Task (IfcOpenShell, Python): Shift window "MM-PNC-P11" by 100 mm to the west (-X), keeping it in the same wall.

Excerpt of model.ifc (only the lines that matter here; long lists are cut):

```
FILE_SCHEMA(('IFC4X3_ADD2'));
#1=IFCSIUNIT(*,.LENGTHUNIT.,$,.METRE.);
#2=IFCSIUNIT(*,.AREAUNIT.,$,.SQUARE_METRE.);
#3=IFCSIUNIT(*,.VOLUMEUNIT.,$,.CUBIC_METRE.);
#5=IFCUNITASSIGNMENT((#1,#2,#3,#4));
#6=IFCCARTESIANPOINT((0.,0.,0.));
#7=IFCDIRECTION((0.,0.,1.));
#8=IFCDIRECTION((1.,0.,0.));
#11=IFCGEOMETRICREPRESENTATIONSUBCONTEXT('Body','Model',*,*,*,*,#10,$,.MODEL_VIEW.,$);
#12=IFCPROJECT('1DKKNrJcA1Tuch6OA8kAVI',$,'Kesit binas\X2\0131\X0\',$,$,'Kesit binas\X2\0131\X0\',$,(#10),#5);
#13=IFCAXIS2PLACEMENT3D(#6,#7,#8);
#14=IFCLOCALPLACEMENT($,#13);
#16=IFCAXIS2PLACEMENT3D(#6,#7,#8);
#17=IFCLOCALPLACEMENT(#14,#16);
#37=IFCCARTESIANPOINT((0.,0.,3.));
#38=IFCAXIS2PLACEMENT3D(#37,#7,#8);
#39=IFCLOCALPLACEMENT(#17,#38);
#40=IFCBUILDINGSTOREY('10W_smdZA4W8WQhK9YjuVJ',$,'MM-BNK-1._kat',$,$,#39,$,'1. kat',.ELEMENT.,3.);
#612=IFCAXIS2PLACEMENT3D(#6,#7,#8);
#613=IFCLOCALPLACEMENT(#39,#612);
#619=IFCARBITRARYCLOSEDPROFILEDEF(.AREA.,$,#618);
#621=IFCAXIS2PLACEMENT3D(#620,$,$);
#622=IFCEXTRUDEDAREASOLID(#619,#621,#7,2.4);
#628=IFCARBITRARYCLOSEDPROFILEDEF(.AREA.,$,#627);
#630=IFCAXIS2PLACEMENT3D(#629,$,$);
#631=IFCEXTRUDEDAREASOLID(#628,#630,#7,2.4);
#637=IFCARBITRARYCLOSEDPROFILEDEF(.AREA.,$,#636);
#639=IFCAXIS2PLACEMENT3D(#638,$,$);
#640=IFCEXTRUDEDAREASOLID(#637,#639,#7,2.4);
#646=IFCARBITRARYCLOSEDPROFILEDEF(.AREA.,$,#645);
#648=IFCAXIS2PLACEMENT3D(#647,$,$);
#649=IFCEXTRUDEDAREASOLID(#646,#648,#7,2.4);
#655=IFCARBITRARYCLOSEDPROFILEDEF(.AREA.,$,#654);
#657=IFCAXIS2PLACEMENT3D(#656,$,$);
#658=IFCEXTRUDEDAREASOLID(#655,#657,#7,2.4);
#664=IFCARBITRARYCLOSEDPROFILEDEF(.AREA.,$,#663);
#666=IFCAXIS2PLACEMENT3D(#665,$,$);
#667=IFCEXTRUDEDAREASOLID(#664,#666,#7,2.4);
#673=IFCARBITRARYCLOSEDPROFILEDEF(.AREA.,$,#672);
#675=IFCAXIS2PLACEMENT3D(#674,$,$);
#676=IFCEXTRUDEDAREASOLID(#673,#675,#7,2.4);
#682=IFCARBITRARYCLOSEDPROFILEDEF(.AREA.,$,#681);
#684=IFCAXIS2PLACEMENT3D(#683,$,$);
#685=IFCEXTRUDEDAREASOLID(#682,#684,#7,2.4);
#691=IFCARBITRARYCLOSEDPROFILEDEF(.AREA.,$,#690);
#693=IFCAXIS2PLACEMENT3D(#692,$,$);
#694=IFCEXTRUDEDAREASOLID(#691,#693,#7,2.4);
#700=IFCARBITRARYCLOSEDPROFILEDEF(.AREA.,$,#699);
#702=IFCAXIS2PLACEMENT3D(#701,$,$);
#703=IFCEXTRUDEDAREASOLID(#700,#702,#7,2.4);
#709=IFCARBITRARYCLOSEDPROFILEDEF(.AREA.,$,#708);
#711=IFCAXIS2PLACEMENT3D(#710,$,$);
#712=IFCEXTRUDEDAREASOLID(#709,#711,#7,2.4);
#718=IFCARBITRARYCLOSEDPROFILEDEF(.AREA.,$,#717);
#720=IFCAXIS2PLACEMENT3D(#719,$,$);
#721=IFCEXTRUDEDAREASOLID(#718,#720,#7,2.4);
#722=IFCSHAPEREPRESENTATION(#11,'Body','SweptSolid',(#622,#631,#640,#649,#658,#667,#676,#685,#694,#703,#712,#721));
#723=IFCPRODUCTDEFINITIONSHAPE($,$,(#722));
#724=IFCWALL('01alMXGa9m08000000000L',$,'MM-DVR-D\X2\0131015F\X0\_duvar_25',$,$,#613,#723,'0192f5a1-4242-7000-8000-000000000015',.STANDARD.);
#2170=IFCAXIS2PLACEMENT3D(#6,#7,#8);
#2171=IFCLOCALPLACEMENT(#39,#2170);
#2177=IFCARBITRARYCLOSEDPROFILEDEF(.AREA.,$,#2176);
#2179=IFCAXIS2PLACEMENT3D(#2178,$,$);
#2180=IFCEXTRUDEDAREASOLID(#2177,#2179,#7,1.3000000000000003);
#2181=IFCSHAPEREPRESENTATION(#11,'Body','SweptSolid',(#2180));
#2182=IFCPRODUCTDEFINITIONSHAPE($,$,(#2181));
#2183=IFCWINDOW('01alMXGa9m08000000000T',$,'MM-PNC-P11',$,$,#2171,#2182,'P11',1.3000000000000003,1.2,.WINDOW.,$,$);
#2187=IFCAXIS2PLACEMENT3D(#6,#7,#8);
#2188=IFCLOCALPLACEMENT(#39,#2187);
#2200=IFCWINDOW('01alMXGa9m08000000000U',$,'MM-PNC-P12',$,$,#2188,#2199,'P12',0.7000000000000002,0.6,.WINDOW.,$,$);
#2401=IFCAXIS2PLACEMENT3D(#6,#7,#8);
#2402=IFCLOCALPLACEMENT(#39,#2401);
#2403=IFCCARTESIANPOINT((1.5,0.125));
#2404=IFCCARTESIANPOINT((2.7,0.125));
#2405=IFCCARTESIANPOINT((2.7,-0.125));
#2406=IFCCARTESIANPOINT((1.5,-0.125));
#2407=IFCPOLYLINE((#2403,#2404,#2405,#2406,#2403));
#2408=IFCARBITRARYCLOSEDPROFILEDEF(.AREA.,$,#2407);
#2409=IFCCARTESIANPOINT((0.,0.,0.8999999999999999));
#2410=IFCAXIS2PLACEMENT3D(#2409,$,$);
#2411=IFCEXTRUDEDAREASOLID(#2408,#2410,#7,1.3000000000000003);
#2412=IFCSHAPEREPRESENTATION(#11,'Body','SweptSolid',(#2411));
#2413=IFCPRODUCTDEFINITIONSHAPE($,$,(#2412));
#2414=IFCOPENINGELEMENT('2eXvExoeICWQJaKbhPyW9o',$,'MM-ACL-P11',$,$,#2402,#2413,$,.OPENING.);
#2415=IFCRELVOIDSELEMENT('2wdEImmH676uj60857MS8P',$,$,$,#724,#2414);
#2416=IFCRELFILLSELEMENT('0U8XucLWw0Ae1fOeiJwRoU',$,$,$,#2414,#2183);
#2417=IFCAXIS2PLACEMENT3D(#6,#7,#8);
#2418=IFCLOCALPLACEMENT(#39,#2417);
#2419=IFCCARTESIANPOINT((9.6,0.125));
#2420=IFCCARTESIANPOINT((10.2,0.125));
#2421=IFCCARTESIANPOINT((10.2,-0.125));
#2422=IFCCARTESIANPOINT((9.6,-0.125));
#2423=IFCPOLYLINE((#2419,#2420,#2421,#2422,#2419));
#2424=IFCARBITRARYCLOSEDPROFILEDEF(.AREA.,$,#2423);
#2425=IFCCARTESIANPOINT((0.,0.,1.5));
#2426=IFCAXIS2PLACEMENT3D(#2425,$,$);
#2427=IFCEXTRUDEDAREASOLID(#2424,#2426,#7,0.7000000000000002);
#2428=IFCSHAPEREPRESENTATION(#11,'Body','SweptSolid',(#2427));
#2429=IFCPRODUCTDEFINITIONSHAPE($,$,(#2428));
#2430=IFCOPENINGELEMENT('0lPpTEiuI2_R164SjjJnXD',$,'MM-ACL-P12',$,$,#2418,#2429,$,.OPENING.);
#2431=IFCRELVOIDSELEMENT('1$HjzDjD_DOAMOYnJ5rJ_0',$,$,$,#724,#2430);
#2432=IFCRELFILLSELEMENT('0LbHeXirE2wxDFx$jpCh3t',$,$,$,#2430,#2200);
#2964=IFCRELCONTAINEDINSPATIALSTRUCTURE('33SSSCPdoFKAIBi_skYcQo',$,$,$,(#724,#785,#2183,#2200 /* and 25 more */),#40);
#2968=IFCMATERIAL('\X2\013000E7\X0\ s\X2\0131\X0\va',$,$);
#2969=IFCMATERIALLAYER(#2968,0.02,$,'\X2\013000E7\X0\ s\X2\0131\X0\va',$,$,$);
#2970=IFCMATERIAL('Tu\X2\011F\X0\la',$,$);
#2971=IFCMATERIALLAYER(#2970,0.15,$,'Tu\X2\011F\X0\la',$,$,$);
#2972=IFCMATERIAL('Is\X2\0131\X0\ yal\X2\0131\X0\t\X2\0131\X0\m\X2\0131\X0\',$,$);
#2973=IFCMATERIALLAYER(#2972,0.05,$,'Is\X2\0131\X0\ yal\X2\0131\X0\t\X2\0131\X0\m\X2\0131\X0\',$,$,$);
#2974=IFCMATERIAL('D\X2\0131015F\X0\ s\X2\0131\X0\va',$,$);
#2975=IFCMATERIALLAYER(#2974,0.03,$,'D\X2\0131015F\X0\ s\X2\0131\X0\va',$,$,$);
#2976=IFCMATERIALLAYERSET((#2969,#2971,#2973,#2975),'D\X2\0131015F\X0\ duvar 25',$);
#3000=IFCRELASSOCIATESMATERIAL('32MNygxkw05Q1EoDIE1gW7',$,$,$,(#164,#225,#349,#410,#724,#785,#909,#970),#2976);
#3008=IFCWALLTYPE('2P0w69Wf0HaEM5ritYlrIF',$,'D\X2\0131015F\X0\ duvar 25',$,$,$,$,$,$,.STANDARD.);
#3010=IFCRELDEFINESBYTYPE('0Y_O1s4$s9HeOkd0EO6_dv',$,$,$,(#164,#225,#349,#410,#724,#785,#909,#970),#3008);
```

```python
import ifcopenshell
import ifcopenshell.api.geometry
import ifcopenshell.util.placement

model = ifcopenshell.open("model.ifc")

window = model.by_guid("01alMXGa9m08000000000T")
opening = window.FillsVoids[0].RelatingOpeningElement
wall = opening.VoidsElements[0].RelatingBuildingElement

wall_matrix = ifcopenshell.util.placement.get_local_placement(wall.ObjectPlacement)
shift = wall_matrix[:3, 0] * -0.1
before = ifcopenshell.util.placement.get_local_placement(window.ObjectPlacement)[:3, 3].copy()

# The window is not placed relative to its opening, so move both.
for product in (opening, window):
    matrix = ifcopenshell.util.placement.get_local_placement(product.ObjectPlacement)
    matrix[:3, 3] += shift
    ifcopenshell.api.geometry.edit_object_placement(model, product=product, matrix=matrix, is_si=False)

after = ifcopenshell.util.placement.get_local_placement(window.ObjectPlacement)[:3, 3]
print("window moved by", (after - before).round(3) + 0.0)

model.write("model_updated.ifc")
```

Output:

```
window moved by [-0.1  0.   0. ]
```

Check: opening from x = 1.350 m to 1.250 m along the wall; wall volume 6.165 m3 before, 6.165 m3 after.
